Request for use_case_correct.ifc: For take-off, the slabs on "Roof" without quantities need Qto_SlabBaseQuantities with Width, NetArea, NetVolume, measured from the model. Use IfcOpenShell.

First a look at what the model holds.

```python
import ifcopenshell
import ifcopenshell.util.element
import ifcopenshell.util.unit

model = ifcopenshell.open("use_case_correct.ifc")
print(model.schema)
for unit_type in ("LENGTHUNIT", "AREAUNIT", "VOLUMEUNIT"):
    print(unit_type, ifcopenshell.util.unit.calculate_unit_scale(model, unit_type))
storey = next(s for s in model.by_type("IfcBuildingStorey") if s.Name == "Roof")
slabs = [e for e in ifcopenshell.util.element.get_decomposition(storey) if e.is_a("IfcSlab")]
for e in sorted(slabs, key=lambda e: e.id()):
    print(e.id(), e.is_a(), e.Name, list(ifcopenshell.util.element.get_psets(e, qtos_only=True)), sep=" | ")
```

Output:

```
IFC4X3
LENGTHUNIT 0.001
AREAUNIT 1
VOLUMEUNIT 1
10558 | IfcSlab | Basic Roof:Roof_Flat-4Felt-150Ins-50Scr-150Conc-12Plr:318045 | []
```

```python
import ifcopenshell
import ifcopenshell.api.pset
import ifcopenshell.geom
import ifcopenshell.util.element
import ifcopenshell.util.shape
import ifcopenshell.util.unit

model = ifcopenshell.open("use_case_correct.ifc")
unit_scale = ifcopenshell.util.unit.calculate_unit_scale(model)
area_scale = ifcopenshell.util.unit.calculate_unit_scale(model, "AREAUNIT")
volume_scale = ifcopenshell.util.unit.calculate_unit_scale(model, "VOLUMEUNIT")
settings = ifcopenshell.geom.settings()

storey = next(s for s in model.by_type("IfcBuildingStorey") if s.Name == "Roof")
slabs = [e for e in ifcopenshell.util.element.get_decomposition(storey) if e.is_a("IfcSlab")]

for e in sorted(slabs, key=lambda e: e.id()):
    if ifcopenshell.util.element.get_psets(e, qtos_only=True, should_inherit=False):
        continue
    # Geometry comes back in metres, in the element's own axes.
    shape = ifcopenshell.geom.create_shape(settings, e)
    values = {
        "Width": ifcopenshell.util.shape.get_z(shape.geometry) / unit_scale,
        "NetArea": ifcopenshell.util.shape.get_footprint_area(shape.geometry) / area_scale,
        "NetVolume": ifcopenshell.util.shape.get_volume(shape.geometry) / volume_scale,
    }
    qto = ifcopenshell.api.pset.add_qto(model, product=e, name="Qto_SlabBaseQuantities")
    ifcopenshell.api.pset.edit_qto(model, qto=qto, properties=values)
    print(e.id(), {k: round(v, 3) for k, v in values.items()})

model.write("use_case_correct_rev.ifc")
```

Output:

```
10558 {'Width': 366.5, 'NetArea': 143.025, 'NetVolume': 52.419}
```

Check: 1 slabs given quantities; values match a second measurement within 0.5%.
